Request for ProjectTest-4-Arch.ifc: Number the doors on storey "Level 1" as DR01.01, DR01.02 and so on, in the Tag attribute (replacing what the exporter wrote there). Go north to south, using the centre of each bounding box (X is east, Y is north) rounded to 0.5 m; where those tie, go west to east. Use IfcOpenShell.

First a look at what the model holds.

```python
import ifcopenshell
import ifcopenshell.util.element
import ifcopenshell.util.placement

model = ifcopenshell.open("ProjectTest-4-Arch.ifc")
print(model.schema)
storey = next(s for s in model.by_type("IfcBuildingStorey") if s.Name == "Level 1")
doors = [e for e in ifcopenshell.util.element.get_decomposition(storey) if e.is_a("IfcDoor")]
for e in sorted(doors, key=lambda e: e.id()):
    origin = ifcopenshell.util.placement.get_local_placement(e.ObjectPlacement)[:3, 3]
    print(e.id(), e.Tag, e.Name, origin.round(2) + 0.0, sep=" | ")
```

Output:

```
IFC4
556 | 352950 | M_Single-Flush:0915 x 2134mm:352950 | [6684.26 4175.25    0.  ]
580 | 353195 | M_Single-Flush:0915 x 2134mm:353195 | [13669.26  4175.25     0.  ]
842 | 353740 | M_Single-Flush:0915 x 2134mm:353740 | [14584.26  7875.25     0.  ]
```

```python
import ifcopenshell
import ifcopenshell.geom
import ifcopenshell.util.element
import ifcopenshell.util.shape

model = ifcopenshell.open("ProjectTest-4-Arch.ifc")
settings = ifcopenshell.geom.settings()
settings.set("use-world-coords", True)


def centre(element):
    shape = ifcopenshell.geom.create_shape(settings, element)
    return ifcopenshell.util.shape.get_bbox_centroid(shape.geometry)


storey = next(s for s in model.by_type("IfcBuildingStorey") if s.Name == "Level 1")
doors = [e for e in ifcopenshell.util.element.get_decomposition(storey) if e.is_a("IfcDoor")]

# Insertion points can sit at a corner or the storey origin, so sort by the geometry (in metres).
centres = {e: centre(e) for e in doors}
doors.sort(key=lambda e: (-round(centres[e][1] / 0.5), centres[e][0]))

for i, e in enumerate(doors, start=1):
    number = f"DR01.{i:02d}"
    e.Tag = number
    print(e.id(), number)

model.write("ProjectTest-4-Arch_updated.ifc")
```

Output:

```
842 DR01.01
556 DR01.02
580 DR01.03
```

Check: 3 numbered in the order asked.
